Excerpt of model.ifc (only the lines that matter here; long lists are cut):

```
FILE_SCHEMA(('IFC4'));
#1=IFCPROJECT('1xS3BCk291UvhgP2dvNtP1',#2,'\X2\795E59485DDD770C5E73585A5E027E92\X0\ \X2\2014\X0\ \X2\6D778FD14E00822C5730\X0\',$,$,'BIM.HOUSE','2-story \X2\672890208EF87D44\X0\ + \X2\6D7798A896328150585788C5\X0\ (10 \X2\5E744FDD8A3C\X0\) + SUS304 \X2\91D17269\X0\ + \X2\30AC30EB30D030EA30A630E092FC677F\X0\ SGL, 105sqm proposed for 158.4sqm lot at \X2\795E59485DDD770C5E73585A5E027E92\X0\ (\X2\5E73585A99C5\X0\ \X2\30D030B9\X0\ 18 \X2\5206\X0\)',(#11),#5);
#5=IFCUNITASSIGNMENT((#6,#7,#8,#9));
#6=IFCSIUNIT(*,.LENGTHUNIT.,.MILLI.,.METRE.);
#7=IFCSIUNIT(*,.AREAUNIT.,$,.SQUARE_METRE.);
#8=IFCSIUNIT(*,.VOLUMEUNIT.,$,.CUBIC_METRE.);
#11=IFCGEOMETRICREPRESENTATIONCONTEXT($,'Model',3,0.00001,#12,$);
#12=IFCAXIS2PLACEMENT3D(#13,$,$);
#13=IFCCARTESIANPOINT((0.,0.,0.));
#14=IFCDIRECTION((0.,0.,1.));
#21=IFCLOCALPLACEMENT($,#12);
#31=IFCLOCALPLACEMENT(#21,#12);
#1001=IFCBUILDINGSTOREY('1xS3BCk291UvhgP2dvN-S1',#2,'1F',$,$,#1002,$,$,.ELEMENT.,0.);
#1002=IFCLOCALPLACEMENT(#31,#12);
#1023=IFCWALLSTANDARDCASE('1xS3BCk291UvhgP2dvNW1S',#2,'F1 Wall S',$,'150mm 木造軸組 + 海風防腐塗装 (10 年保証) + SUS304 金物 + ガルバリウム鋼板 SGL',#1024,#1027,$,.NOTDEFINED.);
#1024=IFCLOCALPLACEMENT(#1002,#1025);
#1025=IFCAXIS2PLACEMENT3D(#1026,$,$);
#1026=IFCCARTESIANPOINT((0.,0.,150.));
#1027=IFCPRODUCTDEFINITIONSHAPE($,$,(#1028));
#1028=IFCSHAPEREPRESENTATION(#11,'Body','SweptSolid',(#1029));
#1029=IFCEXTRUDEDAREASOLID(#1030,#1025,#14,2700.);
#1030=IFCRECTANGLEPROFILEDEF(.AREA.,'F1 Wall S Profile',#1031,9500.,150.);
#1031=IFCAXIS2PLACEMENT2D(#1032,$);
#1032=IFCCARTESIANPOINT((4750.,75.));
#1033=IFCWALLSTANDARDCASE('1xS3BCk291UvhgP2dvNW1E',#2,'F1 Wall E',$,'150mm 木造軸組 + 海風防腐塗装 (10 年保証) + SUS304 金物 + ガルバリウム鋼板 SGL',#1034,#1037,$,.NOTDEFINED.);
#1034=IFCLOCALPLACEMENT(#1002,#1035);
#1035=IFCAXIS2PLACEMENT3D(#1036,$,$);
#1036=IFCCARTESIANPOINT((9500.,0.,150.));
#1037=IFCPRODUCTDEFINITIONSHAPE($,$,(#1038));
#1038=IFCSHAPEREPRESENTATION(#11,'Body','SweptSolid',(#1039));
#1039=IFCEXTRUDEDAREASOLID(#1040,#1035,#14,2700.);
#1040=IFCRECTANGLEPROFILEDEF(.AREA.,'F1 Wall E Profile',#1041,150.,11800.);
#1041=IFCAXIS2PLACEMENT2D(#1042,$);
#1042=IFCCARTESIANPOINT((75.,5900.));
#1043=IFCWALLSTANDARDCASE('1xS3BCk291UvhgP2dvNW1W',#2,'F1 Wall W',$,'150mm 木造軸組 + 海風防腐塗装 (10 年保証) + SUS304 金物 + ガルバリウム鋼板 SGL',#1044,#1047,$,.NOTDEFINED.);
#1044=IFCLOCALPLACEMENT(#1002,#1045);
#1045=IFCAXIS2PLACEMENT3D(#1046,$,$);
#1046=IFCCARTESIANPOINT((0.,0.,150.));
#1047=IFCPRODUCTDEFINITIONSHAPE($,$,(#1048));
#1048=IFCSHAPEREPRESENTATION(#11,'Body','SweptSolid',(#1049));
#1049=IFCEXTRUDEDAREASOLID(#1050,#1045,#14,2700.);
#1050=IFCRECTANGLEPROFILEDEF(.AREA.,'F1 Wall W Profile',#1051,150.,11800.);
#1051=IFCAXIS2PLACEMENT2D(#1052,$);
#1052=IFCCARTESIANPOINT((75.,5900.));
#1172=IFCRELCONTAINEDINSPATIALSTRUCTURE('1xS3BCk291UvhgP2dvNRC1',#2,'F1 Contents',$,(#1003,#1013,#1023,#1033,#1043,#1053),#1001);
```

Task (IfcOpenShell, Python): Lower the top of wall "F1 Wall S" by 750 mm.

```python
import ifcopenshell
import ifcopenshell.geom
import ifcopenshell.util.shape

model = ifcopenshell.open("model.ifc")
settings = ifcopenshell.geom.settings()


def volume(element):
    """Net volume in cubic metres, openings subtracted."""
    shape = ifcopenshell.geom.create_shape(settings, element)
    return ifcopenshell.util.shape.get_volume(shape.geometry)


wall = model.by_id(1023)
before = volume(wall)

body = next(r for r in wall.Representation.Representations if r.RepresentationIdentifier == "Body")
solid = body.Items[0]
old_height = solid.Depth
solid.Depth -= 750.0
after = volume(wall)

print(f"height {old_height:g} -> {solid.Depth:g}, volume {before:.3f} -> {after:.3f} m3")

model.write("model_updated.ifc")
```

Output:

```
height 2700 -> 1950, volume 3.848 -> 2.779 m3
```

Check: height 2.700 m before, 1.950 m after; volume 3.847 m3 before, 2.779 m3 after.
